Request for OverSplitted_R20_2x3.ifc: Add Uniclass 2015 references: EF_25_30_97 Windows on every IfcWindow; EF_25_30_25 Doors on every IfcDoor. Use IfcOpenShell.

First a look at what the model holds.

```python
import ifcopenshell

model = ifcopenshell.open("OverSplitted_R20_2x3.ifc")
print(model.schema)
print("classifications:", [c.Name for c in model.by_type("IfcClassification")])
for ifc_class in ("IfcDoor", "IfcRoof", "IfcStair", "IfcWall", "IfcWindow"):
    print(ifc_class, len(model.by_type(ifc_class)))
```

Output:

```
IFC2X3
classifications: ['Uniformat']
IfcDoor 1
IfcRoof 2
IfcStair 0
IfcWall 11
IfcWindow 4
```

```python
import ifcopenshell
import ifcopenshell.api.classification

model = ifcopenshell.open("OverSplitted_R20_2x3.ifc")

# IFC2X3 requires Source and Edition and has no link from the project to the system.
system = model.create_entity("IfcClassification", Source="NBS", Edition="2015", Name="Uniclass 2015")

codes = {
    "IfcWindow": ("EF_25_30_97", "Windows"),
    "IfcDoor": ("EF_25_30_25", "Doors"),
}
for ifc_class, (code, name) in codes.items():
    products = model.by_type(ifc_class)
    ifcopenshell.api.classification.add_reference(
        model, products=products, classification=system, identification=code, name=name
    )
    print(code, len(products))

model.write("OverSplitted_R20_2x3-out.ifc")
```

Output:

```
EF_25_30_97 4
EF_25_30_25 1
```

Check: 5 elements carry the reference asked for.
